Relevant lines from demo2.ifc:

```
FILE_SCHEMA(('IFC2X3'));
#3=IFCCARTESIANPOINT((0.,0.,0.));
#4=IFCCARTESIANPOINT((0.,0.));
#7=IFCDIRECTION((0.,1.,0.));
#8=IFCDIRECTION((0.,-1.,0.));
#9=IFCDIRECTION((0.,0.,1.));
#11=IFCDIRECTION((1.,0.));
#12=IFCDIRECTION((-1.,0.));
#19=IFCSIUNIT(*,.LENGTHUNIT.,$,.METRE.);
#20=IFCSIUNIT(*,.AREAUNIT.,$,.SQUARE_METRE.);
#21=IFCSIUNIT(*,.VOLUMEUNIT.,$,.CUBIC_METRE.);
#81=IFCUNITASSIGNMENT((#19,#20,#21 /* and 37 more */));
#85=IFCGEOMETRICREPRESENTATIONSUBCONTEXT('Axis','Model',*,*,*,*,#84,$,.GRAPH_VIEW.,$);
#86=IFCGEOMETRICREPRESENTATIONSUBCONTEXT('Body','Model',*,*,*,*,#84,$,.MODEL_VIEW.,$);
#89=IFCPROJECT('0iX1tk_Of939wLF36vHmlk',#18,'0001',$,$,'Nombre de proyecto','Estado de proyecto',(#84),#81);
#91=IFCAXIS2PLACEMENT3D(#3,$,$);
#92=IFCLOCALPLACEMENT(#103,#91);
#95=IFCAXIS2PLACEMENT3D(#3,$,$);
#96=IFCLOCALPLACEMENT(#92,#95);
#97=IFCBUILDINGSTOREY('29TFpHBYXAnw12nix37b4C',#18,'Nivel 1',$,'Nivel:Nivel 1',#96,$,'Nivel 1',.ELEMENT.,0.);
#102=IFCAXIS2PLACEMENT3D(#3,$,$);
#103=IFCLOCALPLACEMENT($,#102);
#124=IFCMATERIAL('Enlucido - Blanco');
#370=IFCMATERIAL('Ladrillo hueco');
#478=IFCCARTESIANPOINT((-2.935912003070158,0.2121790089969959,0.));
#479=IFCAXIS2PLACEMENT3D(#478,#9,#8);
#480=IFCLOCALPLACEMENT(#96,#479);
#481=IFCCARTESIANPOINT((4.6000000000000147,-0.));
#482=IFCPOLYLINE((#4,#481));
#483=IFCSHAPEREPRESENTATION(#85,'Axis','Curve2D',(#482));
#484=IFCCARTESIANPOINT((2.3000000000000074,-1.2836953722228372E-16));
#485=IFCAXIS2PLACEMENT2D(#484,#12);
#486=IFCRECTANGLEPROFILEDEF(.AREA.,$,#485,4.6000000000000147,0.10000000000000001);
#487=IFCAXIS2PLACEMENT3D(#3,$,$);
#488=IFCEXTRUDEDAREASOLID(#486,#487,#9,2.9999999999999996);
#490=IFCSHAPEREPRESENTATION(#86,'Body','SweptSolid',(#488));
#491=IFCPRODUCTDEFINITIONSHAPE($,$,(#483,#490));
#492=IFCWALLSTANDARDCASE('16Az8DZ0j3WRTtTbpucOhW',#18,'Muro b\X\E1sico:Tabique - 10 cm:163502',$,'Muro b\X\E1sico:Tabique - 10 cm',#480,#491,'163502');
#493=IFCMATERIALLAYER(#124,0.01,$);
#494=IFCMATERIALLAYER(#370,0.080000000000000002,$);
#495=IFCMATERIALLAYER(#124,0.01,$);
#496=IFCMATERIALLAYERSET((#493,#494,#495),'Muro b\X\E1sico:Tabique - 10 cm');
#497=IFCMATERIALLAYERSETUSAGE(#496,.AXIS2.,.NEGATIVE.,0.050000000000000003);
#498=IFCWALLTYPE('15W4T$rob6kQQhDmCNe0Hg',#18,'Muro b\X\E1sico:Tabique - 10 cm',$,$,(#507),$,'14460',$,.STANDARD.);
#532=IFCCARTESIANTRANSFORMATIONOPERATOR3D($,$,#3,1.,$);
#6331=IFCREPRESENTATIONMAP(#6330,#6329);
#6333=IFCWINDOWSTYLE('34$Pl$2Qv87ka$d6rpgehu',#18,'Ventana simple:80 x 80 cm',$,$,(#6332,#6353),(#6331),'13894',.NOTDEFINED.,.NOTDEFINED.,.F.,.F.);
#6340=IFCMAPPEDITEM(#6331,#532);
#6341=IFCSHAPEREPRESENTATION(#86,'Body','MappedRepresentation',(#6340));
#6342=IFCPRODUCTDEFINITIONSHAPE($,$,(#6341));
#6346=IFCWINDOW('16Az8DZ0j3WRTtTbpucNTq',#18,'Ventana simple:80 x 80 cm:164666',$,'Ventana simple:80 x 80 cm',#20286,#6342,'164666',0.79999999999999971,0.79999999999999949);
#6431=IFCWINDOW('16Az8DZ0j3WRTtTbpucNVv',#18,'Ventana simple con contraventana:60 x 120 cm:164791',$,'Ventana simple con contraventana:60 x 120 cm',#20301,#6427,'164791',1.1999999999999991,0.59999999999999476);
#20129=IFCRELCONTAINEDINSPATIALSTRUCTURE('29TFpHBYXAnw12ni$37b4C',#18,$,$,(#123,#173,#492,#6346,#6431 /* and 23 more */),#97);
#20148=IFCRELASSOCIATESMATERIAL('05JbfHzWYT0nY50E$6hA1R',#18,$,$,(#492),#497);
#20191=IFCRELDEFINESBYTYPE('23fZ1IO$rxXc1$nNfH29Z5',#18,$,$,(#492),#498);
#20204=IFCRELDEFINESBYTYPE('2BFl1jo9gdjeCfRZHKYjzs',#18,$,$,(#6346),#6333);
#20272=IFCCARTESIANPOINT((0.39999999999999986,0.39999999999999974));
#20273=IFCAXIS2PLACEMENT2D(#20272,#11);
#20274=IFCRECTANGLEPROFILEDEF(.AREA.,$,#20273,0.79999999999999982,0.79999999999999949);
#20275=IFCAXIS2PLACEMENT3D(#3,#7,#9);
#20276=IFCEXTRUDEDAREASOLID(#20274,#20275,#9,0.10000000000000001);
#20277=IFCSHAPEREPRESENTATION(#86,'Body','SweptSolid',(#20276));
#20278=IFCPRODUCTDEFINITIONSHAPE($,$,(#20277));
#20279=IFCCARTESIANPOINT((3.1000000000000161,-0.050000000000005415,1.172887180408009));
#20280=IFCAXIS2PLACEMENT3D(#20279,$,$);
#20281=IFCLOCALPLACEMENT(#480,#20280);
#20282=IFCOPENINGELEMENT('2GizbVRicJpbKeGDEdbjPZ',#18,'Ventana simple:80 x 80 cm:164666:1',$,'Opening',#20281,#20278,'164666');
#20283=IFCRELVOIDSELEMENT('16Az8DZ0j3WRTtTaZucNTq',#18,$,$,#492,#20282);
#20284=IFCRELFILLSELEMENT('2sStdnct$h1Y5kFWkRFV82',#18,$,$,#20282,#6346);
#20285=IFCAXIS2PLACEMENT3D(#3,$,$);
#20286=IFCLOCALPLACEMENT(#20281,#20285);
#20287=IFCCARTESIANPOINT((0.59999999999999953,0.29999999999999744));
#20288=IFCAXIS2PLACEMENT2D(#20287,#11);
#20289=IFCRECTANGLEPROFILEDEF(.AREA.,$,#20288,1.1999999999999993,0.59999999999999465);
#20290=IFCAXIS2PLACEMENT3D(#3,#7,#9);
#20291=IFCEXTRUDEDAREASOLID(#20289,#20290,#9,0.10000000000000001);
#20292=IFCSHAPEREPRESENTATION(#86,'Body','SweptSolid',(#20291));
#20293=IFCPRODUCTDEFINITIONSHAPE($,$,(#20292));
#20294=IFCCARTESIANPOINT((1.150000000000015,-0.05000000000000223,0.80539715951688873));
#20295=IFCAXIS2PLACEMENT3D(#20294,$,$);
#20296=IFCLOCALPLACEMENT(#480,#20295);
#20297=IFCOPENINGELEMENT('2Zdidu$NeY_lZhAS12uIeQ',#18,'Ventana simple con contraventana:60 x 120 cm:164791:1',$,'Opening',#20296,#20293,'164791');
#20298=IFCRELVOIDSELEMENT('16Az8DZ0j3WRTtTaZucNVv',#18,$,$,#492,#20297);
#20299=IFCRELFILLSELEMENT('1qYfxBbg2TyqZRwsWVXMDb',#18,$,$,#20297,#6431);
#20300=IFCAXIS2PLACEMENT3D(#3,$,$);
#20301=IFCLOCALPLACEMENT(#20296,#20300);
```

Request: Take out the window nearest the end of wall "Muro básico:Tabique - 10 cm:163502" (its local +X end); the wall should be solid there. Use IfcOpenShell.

```python
import ifcopenshell
import ifcopenshell.api.feature
import ifcopenshell.api.root
import ifcopenshell.geom
import ifcopenshell.util.shape

model = ifcopenshell.open("demo2.ifc")
settings = ifcopenshell.geom.settings()


def volume(element):
    """Net volume in cubic metres, openings subtracted."""
    shape = ifcopenshell.geom.create_shape(settings, element)
    return ifcopenshell.util.shape.get_volume(shape.geometry)


window = model.by_guid("16Az8DZ0j3WRTtTbpucNTq")
opening = window.FillsVoids[0].RelatingOpeningElement
wall = opening.VoidsElements[0].RelatingBuildingElement
before = volume(wall)

ifcopenshell.api.root.remove_product(model, product=window)
ifcopenshell.api.feature.remove_feature(model, feature=opening)

after = volume(wall)

print(f"wall volume {before:.3f} -> {after:.3f} m3")

model.write("demo2_rev.ifc")
```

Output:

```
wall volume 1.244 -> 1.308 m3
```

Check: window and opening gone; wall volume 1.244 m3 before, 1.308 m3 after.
